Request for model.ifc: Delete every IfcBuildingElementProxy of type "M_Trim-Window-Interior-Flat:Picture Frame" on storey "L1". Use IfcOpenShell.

First a look at what the model holds.

```python
import ifcopenshell
import ifcopenshell.util.element

model = ifcopenshell.open("model.ifc")
print(model.schema)
storey = next(s for s in model.by_type("IfcBuildingStorey") if s.Name == "L1")
proxies = [e for e in ifcopenshell.util.element.get_decomposition(storey) if e.is_a("IfcBuildingElementProxy")]
seen = {}
for e in proxies:
    element_type = ifcopenshell.util.element.get_type(e)
    name = element_type.Name if element_type not in (None, e) else None
    seen[name] = seen.get(name, 0) + 1
for name, count in sorted(seen.items(), key=str):
    print(count, "x", name)
```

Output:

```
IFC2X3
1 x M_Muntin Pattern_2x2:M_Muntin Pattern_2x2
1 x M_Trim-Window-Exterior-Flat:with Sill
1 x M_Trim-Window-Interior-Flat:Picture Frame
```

```python
import ifcopenshell
import ifcopenshell.api.root
import ifcopenshell.util.element

model = ifcopenshell.open("model.ifc")

storey = next(s for s in model.by_type("IfcBuildingStorey") if s.Name == "L1")
proxies = [e for e in ifcopenshell.util.element.get_decomposition(storey) if e.is_a("IfcBuildingElementProxy")]
targets = [e for e in proxies if (t := ifcopenshell.util.element.get_type(e)) not in (None, e) and t.Name == "M_Trim-Window-Interior-Flat:Picture Frame"]

for e in targets:
    ifcopenshell.api.root.remove_product(model, product=e)
print(len(targets), "removed")

model.write("model-out.ifc")
```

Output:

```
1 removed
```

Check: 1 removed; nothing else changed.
